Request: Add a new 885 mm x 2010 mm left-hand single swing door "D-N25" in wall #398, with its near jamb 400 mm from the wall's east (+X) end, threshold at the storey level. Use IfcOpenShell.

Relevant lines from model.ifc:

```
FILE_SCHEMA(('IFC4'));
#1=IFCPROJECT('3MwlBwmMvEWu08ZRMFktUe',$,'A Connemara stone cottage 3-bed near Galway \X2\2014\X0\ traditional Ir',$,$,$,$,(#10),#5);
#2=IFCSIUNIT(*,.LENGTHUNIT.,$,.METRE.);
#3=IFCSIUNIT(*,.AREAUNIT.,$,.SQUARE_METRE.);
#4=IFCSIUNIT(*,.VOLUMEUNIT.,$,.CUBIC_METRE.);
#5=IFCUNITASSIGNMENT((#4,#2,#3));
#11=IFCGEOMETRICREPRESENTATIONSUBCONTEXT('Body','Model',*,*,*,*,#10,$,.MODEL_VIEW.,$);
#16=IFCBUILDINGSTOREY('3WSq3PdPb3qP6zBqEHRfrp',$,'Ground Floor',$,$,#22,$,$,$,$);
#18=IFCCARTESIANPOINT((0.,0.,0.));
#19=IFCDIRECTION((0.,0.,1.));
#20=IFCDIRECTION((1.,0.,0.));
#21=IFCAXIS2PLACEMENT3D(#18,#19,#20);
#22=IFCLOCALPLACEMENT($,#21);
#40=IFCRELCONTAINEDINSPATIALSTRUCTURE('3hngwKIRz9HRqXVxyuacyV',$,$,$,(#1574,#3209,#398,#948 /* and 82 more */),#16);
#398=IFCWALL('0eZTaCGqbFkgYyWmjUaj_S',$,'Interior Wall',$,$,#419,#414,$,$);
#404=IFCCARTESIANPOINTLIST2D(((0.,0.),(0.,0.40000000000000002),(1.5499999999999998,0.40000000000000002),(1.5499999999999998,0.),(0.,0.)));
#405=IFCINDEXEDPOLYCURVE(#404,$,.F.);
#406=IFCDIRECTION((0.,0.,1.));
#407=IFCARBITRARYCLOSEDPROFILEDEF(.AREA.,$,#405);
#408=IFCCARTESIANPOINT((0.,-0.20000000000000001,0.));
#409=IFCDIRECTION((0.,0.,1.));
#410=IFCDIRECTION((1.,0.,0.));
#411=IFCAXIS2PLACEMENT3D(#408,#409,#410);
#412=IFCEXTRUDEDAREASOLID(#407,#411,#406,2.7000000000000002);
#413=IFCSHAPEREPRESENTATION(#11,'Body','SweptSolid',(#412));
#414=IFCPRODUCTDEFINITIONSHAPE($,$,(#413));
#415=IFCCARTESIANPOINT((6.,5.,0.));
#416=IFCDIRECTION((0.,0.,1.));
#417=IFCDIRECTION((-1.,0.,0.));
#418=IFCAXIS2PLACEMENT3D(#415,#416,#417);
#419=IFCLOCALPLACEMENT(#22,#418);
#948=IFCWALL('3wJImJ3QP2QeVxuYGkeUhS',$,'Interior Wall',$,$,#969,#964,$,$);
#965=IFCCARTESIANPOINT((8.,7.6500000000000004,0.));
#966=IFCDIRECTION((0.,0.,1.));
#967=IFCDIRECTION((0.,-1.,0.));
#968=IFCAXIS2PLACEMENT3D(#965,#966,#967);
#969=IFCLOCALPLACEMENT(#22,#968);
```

```python
import numpy as np
import ifcopenshell
import ifcopenshell.api.feature
import ifcopenshell.api.geometry
import ifcopenshell.api.root
import ifcopenshell.api.spatial
import ifcopenshell.geom
import ifcopenshell.util.element
import ifcopenshell.util.placement
import ifcopenshell.util.representation
import ifcopenshell.util.shape
import ifcopenshell.util.unit

model = ifcopenshell.open("model.ifc")
unit_scale = ifcopenshell.util.unit.calculate_unit_scale(model)
settings = ifcopenshell.geom.settings()


def volume(element):
    """Net volume in cubic metres, openings subtracted."""
    shape = ifcopenshell.geom.create_shape(settings, element)
    return ifcopenshell.util.shape.get_volume(shape.geometry)


wall = model.by_id(398)
storey = ifcopenshell.util.element.get_container(wall, ifc_class="IfcBuildingStorey")
context = ifcopenshell.util.representation.get_context(model, "Model", "Body", "MODEL_VIEW")
before = volume(wall)

width, height, from_end, sill = 0.885, 2.01, 0.4, 0.0  # metres

# The wall runs along its own X axis, and the end named is its -X end.
wall_shape = ifcopenshell.geom.create_shape(settings, wall)
x, y, z = ifcopenshell.util.shape.get_vertices(wall_shape.geometry).T
start = x.min() + from_end
face, thickness = float(y.min()), float(y.max() - y.min())
wall_matrix = ifcopenshell.util.placement.get_local_placement(wall.ObjectPlacement)
level = ifcopenshell.util.placement.get_local_placement(storey.ObjectPlacement)[2, 3]


def in_wall(x, y):
    """Placement at x, y metres in the wall's axes, at sill height."""
    matrix = wall_matrix.copy()
    matrix[:, 3] = wall_matrix @ np.array([x / unit_scale, y / unit_scale, 0.0, 1.0])
    matrix[2, 3] = level + sill / unit_scale
    return matrix


# Opening: a box that overshoots both wall faces by 50 mm.
opening = ifcopenshell.api.root.create_entity(model, ifc_class="IfcOpeningElement", predefined_type="OPENING")
box = ifcopenshell.api.geometry.add_wall_representation(
    model, context=context, length=width, height=height, thickness=thickness + 0.1
)
ifcopenshell.api.geometry.assign_representation(model, product=opening, representation=box)
ifcopenshell.api.geometry.edit_object_placement(model, product=opening, matrix=in_wall(start, face - 0.05), is_si=False)
ifcopenshell.api.feature.add_feature(model, feature=opening, element=wall)

door = ifcopenshell.api.root.create_entity(model, ifc_class="IfcDoor", name="D-N25", predefined_type="DOOR")
door.OverallWidth, door.OverallHeight = width / unit_scale, height / unit_scale
door.OperationType = "SINGLE_SWING_LEFT"
body = ifcopenshell.api.geometry.add_door_representation(
    model,
    context=context,
    overall_width=door.OverallWidth,
    overall_height=door.OverallHeight,
    operation_type="SINGLE_SWING_LEFT",
    lining_properties={"LiningDepth": thickness / unit_scale, "ThresholdDepth": thickness / unit_scale},
)
ifcopenshell.api.geometry.assign_representation(model, product=door, representation=body)
ifcopenshell.api.spatial.assign_container(model, products=[door], relating_structure=storey)
ifcopenshell.api.feature.add_filling(model, opening=opening, element=door)

# The lining spans the wall, so the door starts at the wall face.
ifcopenshell.api.geometry.edit_object_placement(model, product=door, matrix=in_wall(start, face), is_si=False)

after = volume(wall)

print(f"wall volume {before:.3f} -> {after:.3f} m3")

model.write("model_v2.ifc")
```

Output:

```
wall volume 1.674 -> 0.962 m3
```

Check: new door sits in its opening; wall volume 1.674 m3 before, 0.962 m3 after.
